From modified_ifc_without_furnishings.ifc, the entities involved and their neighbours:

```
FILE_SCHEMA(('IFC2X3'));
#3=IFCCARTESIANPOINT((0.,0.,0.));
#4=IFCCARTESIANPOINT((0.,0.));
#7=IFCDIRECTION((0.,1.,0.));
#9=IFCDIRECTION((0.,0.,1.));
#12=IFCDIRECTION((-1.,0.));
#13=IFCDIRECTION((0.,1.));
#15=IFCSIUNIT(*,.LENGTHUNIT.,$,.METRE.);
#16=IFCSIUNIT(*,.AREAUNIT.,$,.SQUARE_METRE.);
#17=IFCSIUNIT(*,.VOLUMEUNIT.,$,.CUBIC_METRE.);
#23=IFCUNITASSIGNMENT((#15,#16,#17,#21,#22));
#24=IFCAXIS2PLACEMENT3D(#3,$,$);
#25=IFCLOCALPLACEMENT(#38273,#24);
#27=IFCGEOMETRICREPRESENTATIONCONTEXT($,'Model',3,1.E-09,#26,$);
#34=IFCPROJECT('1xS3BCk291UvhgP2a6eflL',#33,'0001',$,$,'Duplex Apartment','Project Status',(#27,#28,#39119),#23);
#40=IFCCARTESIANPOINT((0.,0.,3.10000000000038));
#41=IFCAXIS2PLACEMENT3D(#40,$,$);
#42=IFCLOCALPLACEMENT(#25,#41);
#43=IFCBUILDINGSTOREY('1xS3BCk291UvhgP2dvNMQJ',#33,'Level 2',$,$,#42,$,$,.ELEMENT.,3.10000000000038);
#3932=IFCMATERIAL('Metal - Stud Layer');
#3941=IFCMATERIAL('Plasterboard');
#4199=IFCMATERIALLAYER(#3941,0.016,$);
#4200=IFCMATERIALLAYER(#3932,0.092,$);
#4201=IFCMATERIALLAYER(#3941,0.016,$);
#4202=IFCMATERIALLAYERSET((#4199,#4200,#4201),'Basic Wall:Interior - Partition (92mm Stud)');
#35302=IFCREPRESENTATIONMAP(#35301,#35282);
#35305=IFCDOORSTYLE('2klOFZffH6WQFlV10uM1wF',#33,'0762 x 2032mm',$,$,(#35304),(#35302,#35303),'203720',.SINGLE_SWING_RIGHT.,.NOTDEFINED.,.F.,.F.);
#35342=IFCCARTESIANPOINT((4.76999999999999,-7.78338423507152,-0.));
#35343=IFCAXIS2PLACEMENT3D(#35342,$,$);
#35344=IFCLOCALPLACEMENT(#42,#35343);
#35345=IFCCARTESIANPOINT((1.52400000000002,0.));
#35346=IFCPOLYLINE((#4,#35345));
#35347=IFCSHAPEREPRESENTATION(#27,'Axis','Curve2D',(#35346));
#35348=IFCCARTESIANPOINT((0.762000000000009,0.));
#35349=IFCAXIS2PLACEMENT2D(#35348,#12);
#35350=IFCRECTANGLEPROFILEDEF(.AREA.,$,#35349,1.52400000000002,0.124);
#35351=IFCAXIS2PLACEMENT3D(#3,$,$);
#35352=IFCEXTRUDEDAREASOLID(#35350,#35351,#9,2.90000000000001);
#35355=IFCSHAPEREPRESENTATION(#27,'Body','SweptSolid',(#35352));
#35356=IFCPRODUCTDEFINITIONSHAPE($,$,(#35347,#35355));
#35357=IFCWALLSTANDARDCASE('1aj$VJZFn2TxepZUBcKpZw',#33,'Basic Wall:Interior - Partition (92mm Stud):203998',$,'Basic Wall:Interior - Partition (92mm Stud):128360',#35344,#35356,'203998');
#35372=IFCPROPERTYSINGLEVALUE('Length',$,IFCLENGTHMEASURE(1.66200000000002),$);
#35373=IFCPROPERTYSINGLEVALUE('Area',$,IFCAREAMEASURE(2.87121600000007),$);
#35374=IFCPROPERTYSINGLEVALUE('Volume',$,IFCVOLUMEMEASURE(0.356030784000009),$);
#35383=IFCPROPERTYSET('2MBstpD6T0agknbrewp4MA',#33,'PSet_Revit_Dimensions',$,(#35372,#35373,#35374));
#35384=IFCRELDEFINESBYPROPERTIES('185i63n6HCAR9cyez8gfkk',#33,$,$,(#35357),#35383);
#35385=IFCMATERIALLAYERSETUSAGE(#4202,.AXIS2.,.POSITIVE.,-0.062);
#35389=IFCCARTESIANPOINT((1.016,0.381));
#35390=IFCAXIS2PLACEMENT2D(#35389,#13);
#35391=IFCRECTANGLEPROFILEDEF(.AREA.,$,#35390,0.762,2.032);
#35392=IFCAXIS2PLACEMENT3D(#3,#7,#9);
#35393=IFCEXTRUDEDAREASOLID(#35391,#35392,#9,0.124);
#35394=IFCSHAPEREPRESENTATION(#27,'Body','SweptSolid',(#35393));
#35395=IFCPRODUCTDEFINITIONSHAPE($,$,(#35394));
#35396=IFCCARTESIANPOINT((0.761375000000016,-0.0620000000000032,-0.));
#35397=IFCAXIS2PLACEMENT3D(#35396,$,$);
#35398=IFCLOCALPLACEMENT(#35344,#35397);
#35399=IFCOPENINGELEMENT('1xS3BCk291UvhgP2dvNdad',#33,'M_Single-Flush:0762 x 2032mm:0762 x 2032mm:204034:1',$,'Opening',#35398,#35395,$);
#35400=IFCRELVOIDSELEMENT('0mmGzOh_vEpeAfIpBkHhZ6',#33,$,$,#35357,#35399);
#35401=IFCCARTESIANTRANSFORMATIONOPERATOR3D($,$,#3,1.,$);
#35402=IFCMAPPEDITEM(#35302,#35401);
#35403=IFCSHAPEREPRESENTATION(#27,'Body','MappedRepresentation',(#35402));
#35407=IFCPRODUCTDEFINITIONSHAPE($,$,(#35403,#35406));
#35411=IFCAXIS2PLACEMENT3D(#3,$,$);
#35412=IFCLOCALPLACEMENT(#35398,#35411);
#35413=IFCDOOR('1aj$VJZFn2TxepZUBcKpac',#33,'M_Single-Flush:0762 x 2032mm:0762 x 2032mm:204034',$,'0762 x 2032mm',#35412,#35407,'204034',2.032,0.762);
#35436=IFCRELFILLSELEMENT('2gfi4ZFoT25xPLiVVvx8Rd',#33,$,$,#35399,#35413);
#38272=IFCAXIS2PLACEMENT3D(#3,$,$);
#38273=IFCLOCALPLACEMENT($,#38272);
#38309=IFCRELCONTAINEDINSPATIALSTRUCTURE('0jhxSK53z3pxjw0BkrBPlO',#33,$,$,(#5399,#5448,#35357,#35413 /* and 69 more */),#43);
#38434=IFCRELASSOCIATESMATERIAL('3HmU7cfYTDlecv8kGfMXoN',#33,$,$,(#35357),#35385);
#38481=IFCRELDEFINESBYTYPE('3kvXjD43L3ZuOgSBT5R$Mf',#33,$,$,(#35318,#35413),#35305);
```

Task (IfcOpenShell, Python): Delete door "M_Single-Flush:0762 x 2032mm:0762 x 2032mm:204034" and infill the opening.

```python
import ifcopenshell
import ifcopenshell.api.feature
import ifcopenshell.api.pset
import ifcopenshell.api.root
import ifcopenshell.geom
import ifcopenshell.util.element
import ifcopenshell.util.shape
import ifcopenshell.util.unit

model = ifcopenshell.open("modified_ifc_without_furnishings.ifc")
area_scale = ifcopenshell.util.unit.calculate_unit_scale(model, "AREAUNIT")
volume_scale = ifcopenshell.util.unit.calculate_unit_scale(model, "VOLUMEUNIT")
settings = ifcopenshell.geom.settings()


def volume(element):
    """Net volume in cubic metres, openings subtracted."""
    shape = ifcopenshell.geom.create_shape(settings, element)
    return ifcopenshell.util.shape.get_volume(shape.geometry)


door = model.by_guid("1aj$VJZFn2TxepZUBcKpac")
opening = door.FillsVoids[0].RelatingOpeningElement
wall = opening.VoidsElements[0].RelatingBuildingElement
before = volume(wall)

ifcopenshell.api.root.remove_product(model, product=door)
ifcopenshell.api.feature.remove_feature(model, feature=opening)

after = volume(wall)
thickness = 0.124  # wall thickness in metres

# Update the wall's stored quantities.
pset = model.by_id(ifcopenshell.util.element.get_pset(wall, "PSet_Revit_Dimensions", should_inherit=False)["id"])
ifcopenshell.api.pset.edit_pset(model, pset=pset, properties={
    "Area": model.create_entity("IfcAreaMeasure", after / thickness / area_scale),
    "Volume": model.create_entity("IfcVolumeMeasure", after / volume_scale),
})

print(f"wall volume {before:.3f} -> {after:.3f} m3")

model.write("modified_ifc_without_furnishings_rev.ifc")
```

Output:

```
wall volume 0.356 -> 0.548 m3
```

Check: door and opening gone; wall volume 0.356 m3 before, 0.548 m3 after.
